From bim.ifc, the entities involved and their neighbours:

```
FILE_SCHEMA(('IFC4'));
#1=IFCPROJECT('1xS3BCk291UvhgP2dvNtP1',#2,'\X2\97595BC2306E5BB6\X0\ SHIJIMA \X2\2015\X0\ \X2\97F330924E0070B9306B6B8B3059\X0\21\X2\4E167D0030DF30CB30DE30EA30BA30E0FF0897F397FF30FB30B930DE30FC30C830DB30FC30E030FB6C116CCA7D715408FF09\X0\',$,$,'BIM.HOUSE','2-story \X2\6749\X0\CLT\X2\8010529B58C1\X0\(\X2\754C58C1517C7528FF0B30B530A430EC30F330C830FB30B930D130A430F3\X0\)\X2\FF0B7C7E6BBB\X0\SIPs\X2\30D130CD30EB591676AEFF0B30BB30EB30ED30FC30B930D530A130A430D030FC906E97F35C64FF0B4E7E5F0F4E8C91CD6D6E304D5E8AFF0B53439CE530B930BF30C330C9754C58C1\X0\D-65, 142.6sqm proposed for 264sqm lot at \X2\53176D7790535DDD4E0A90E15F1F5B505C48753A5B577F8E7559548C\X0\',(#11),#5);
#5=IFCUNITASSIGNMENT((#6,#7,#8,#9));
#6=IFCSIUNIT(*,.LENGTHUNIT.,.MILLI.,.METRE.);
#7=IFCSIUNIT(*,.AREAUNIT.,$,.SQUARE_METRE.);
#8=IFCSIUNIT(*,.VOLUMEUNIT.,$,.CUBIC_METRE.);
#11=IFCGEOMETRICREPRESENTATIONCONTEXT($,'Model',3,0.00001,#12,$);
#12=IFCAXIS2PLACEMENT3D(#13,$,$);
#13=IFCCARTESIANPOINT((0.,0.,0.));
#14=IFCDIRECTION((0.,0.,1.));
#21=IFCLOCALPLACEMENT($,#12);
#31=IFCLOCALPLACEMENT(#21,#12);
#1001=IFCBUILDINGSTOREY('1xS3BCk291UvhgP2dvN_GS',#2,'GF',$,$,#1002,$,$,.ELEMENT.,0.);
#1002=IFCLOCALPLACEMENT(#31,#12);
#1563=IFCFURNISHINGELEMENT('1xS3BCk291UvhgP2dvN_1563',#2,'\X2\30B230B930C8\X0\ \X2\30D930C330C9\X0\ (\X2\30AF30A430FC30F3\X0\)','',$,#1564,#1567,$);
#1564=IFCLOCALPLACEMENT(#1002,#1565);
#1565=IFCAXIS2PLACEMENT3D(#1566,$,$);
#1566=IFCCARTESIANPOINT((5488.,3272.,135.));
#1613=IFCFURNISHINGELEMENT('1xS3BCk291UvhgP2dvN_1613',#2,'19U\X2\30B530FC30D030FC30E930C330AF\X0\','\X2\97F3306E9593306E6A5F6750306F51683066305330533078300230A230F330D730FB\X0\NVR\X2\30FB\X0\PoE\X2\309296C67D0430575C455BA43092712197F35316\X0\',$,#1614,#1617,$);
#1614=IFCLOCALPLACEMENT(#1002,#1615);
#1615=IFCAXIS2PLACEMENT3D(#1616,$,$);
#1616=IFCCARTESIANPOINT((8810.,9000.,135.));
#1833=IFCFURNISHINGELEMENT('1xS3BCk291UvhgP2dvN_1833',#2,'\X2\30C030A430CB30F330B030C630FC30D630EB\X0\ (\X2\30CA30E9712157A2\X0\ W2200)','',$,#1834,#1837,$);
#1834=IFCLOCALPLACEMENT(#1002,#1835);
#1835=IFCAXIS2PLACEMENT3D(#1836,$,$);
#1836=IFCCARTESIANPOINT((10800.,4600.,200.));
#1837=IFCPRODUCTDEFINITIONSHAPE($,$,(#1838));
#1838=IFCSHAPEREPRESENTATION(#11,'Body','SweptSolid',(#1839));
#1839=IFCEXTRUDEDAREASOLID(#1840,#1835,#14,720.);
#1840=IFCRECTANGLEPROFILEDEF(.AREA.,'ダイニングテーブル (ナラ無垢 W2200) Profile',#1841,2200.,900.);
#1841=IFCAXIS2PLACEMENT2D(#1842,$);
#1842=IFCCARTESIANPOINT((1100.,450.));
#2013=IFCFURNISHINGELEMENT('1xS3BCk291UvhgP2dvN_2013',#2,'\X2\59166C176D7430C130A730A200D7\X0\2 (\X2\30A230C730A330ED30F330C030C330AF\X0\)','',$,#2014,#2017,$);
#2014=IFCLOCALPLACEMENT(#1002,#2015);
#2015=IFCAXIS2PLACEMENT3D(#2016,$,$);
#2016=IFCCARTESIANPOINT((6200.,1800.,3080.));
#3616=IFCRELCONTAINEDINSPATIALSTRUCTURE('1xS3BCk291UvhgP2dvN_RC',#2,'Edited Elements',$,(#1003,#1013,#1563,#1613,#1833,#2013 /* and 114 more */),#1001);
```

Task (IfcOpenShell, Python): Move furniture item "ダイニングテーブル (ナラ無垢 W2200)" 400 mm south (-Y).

```python
import ifcopenshell
import ifcopenshell.api.geometry
import ifcopenshell.util.placement
import ifcopenshell.util.unit

model = ifcopenshell.open("bim.ifc")
unit_scale = ifcopenshell.util.unit.calculate_unit_scale(model)

item = model.by_guid("1xS3BCk291UvhgP2dvN_1833")
matrix = ifcopenshell.util.placement.get_local_placement(item.ObjectPlacement)
matrix[1, 3] -= 0.4 / unit_scale
ifcopenshell.api.geometry.edit_object_placement(model, product=item, matrix=matrix, is_si=False)

print(ifcopenshell.util.placement.get_local_placement(item.ObjectPlacement).round(3) + 0.0)

model.write("bim_updated.ifc")
```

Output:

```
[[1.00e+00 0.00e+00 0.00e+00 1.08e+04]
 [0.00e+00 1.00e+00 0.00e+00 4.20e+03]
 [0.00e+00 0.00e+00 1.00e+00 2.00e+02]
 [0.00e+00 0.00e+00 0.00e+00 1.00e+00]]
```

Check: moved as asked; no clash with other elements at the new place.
